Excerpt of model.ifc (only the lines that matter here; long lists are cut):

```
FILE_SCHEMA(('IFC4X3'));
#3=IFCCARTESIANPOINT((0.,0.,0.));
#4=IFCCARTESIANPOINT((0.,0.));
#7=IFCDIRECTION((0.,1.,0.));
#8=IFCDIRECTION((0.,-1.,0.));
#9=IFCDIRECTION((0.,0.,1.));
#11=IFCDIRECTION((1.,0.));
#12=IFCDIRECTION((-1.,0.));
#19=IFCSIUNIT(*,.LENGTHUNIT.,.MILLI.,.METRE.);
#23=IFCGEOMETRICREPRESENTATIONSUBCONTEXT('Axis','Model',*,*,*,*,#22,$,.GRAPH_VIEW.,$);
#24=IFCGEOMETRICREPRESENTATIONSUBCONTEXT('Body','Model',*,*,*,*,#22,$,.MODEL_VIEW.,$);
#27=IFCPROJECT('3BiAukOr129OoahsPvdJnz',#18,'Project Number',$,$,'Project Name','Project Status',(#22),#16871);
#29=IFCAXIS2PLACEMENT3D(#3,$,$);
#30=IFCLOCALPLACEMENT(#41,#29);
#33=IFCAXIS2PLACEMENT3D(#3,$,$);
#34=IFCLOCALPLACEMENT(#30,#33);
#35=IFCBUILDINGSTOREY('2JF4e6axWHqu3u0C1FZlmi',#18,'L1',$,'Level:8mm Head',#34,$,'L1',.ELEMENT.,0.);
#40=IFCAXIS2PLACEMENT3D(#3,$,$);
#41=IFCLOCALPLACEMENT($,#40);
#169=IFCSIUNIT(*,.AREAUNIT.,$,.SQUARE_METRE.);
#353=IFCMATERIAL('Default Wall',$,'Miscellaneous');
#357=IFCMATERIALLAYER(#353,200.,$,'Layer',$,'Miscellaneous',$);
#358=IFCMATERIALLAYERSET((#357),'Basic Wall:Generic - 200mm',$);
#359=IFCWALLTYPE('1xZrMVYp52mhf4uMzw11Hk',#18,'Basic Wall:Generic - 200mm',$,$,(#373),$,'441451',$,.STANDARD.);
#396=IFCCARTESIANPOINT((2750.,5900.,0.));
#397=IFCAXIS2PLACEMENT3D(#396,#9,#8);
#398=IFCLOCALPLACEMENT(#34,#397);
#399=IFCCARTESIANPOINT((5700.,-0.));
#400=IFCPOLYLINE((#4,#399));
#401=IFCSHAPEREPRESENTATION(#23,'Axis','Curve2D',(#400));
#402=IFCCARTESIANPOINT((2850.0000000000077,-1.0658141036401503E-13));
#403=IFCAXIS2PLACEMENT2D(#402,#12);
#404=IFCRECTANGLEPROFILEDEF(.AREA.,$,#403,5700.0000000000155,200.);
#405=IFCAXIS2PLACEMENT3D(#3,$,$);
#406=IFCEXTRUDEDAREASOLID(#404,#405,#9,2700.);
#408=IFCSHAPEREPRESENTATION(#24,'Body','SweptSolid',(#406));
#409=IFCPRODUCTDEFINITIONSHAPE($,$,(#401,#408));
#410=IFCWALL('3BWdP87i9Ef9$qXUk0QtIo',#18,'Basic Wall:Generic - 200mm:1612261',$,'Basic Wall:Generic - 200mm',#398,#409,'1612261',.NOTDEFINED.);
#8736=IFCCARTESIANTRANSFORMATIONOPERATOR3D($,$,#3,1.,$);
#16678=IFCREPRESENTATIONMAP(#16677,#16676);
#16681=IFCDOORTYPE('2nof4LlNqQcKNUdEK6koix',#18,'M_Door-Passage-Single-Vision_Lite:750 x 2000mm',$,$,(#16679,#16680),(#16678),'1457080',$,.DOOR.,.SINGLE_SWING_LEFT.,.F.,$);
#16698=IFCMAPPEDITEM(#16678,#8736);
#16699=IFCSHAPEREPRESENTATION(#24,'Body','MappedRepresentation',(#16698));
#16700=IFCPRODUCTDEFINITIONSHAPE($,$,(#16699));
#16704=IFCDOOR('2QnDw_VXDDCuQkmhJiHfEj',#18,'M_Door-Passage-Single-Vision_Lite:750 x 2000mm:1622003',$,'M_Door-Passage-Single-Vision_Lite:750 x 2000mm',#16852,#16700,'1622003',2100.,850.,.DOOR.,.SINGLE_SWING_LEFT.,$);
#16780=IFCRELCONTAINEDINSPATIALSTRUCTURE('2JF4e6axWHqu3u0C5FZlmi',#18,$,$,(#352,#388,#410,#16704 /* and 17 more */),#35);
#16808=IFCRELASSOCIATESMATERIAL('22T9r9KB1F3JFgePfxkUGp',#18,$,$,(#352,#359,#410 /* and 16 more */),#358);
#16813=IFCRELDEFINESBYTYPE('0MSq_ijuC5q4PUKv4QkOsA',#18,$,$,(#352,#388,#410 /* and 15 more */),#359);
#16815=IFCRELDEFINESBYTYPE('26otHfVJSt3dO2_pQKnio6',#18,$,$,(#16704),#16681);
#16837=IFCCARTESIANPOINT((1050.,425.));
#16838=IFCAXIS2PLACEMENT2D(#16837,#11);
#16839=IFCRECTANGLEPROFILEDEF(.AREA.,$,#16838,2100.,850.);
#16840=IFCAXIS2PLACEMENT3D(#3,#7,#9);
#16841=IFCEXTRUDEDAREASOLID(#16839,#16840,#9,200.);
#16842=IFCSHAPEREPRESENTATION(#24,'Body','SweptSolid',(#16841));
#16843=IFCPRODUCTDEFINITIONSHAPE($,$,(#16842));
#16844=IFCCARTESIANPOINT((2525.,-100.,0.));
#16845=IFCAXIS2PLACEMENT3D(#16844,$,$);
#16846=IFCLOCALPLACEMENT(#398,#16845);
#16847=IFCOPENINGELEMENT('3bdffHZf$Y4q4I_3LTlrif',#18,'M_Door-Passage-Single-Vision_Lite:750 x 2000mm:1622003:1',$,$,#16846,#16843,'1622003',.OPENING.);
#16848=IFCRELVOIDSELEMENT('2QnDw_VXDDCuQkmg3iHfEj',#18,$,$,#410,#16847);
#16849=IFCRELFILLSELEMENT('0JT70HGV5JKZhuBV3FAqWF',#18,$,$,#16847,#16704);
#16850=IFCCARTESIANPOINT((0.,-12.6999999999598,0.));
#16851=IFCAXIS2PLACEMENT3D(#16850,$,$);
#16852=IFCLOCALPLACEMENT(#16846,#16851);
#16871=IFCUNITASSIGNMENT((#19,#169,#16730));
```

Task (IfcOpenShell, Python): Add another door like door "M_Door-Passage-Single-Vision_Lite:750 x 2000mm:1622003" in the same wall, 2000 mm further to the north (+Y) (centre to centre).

```python
import ifcopenshell
import ifcopenshell.api.feature
import ifcopenshell.api.geometry
import ifcopenshell.api.root
import ifcopenshell.geom
import ifcopenshell.util.element
import ifcopenshell.util.placement
import ifcopenshell.util.shape
import ifcopenshell.util.unit

model = ifcopenshell.open("model.ifc")
unit_scale = ifcopenshell.util.unit.calculate_unit_scale(model)
settings = ifcopenshell.geom.settings()


def volume(element):
    """Net volume in cubic metres, openings subtracted."""
    shape = ifcopenshell.geom.create_shape(settings, element)
    return ifcopenshell.util.shape.get_volume(shape.geometry)


def reuse_history(source, copy):
    """copy_class also copies each property set's owner history, people and application; keep the originals."""
    for rel in copy.IsDefinedBy:
        if rel.is_a("IfcRelDefinesByProperties") and (history := rel.RelatingPropertyDefinition.OwnerHistory):
            rel.RelatingPropertyDefinition.OwnerHistory = source.OwnerHistory
            ifcopenshell.util.element.remove_deep2(model, history)


door = model.by_guid("2QnDw_VXDDCuQkmhJiHfEj")
opening = door.FillsVoids[0].RelatingOpeningElement
wall = opening.VoidsElements[0].RelatingBuildingElement
before = volume(wall)
shift = ifcopenshell.util.placement.get_local_placement(wall.ObjectPlacement)[:3, 0] * -2 / unit_scale

# copy_class copies the void relationship, type, container and properties, but no geometry.
new_opening = ifcopenshell.api.root.copy_class(model, product=opening)
new_opening.Representation = ifcopenshell.util.element.copy_deep(
    model, opening.Representation, exclude=["IfcGeometricRepresentationContext", "IfcRepresentationMap"]
)
new_opening.Name = "M_Door-Passage-Single-Vision_Lite:750 x 2000mm"
new_opening.Tag = None
new_door = ifcopenshell.api.root.copy_class(model, product=door)
new_door.Representation = ifcopenshell.util.element.copy_deep(
    model, door.Representation, exclude=["IfcGeometricRepresentationContext", "IfcRepresentationMap"]
)
new_door.Name = "M_Door-Passage-Single-Vision_Lite:750 x 2000mm"
new_door.Tag = None
reuse_history(door, new_door)
ifcopenshell.api.feature.add_filling(model, opening=new_opening, element=new_door)

for old, new in ((opening, new_opening), (door, new_door)):
    matrix = ifcopenshell.util.placement.get_local_placement(old.ObjectPlacement)
    matrix[:3, 3] += shift
    ifcopenshell.api.geometry.edit_object_placement(model, product=new, matrix=matrix, is_si=False)

after = volume(wall)

print(f"wall volume {before:.3f} -> {after:.3f} m3")

model.write("model_updated.ifc")
```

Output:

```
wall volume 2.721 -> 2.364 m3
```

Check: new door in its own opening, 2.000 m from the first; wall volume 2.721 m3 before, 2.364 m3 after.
